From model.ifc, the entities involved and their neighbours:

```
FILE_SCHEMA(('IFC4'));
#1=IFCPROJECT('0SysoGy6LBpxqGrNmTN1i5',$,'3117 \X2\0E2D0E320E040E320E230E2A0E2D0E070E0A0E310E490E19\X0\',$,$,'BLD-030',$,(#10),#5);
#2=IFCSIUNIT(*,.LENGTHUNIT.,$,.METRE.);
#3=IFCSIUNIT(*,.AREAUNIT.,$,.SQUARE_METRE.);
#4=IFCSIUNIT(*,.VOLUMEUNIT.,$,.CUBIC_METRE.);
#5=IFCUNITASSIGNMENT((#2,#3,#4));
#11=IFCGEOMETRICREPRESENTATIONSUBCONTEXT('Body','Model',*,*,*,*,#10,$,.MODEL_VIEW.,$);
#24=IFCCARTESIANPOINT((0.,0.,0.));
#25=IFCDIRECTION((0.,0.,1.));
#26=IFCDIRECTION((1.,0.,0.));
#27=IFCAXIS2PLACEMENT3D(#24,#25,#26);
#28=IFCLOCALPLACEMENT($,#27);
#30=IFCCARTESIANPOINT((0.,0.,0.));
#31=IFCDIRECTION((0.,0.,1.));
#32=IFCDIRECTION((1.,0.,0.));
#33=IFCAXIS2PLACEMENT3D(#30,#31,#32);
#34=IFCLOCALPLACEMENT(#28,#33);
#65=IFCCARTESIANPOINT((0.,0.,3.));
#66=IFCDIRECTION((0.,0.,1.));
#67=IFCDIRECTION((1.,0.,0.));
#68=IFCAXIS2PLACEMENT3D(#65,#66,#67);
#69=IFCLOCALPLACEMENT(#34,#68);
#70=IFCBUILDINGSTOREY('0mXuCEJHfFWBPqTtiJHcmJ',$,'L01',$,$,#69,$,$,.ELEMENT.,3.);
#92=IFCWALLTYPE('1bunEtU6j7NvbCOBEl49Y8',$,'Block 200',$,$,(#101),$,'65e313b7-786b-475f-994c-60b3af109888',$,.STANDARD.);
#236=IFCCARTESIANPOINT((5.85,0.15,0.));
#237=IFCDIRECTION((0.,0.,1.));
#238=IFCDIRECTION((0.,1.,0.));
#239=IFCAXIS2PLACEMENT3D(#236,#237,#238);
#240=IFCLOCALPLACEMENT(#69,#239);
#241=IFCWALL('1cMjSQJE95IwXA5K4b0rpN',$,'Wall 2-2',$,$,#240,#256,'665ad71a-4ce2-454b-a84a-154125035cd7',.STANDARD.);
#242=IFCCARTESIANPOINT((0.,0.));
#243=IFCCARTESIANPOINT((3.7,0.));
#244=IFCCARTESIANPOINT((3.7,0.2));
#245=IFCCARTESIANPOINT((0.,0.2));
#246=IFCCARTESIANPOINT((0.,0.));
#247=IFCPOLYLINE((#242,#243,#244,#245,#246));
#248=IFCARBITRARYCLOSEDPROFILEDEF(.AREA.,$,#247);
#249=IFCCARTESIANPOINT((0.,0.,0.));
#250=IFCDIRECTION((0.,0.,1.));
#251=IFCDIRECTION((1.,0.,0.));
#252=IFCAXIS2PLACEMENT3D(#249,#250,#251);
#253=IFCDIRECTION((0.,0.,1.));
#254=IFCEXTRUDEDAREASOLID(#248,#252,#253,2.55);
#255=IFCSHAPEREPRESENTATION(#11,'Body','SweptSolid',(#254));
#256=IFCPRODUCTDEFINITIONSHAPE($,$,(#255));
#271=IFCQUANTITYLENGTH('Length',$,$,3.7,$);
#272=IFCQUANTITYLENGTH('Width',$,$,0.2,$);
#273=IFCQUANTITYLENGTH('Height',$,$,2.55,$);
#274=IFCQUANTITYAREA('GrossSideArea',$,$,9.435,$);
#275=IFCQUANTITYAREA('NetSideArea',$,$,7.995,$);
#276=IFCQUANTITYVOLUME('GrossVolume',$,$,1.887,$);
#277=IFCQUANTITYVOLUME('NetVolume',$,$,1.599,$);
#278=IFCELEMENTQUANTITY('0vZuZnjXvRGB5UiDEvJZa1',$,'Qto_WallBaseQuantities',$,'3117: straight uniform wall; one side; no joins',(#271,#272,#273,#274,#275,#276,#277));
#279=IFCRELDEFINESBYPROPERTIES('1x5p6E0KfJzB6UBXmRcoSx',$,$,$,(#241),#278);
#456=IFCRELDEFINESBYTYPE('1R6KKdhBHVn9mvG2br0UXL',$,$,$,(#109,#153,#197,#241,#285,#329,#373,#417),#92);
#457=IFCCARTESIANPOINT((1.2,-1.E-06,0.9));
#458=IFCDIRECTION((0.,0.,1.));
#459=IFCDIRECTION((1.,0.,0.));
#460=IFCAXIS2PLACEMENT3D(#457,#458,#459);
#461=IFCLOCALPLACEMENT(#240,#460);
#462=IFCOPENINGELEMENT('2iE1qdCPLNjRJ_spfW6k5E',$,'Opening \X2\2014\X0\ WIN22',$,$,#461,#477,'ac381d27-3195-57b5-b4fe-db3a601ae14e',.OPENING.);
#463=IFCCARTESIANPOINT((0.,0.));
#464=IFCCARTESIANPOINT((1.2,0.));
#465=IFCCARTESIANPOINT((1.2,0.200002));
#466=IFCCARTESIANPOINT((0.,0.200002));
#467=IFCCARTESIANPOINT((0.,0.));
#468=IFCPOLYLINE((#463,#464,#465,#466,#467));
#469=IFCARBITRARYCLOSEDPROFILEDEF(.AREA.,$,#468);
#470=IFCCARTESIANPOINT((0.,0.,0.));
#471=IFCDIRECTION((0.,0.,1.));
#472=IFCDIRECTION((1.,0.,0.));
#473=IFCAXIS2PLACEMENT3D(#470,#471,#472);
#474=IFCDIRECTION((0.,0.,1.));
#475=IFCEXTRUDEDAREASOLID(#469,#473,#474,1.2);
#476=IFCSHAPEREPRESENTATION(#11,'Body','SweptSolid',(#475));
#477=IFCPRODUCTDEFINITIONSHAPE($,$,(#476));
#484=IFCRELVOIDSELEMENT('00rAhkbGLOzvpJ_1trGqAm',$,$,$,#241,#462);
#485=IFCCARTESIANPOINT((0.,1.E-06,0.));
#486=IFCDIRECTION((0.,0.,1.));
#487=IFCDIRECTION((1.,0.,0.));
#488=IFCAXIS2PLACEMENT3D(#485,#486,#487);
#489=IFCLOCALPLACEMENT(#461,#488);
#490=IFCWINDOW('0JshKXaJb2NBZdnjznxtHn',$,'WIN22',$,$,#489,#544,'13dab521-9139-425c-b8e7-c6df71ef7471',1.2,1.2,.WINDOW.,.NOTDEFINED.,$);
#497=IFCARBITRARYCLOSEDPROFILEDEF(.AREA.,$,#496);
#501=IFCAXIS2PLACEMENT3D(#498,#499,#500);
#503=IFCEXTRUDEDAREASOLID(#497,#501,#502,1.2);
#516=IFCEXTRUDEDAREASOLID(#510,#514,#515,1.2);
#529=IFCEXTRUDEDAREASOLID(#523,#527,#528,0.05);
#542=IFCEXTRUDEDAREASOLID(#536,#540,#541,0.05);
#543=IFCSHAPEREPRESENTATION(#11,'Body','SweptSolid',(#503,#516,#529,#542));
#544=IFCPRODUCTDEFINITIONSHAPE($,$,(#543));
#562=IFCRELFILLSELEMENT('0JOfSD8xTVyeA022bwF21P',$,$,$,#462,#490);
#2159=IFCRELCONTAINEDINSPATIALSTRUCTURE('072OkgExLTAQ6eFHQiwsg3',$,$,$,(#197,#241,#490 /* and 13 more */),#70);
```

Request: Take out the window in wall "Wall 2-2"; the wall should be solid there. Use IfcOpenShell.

```python
import ifcopenshell
import ifcopenshell.api.feature
import ifcopenshell.api.pset
import ifcopenshell.api.root
import ifcopenshell.geom
import ifcopenshell.util.element
import ifcopenshell.util.shape
import ifcopenshell.util.unit

model = ifcopenshell.open("model.ifc")
area_scale = ifcopenshell.util.unit.calculate_unit_scale(model, "AREAUNIT")
volume_scale = ifcopenshell.util.unit.calculate_unit_scale(model, "VOLUMEUNIT")
settings = ifcopenshell.geom.settings()


def volume(element):
    """Net volume in cubic metres, openings subtracted."""
    shape = ifcopenshell.geom.create_shape(settings, element)
    return ifcopenshell.util.shape.get_volume(shape.geometry)


window = model.by_id(490)
opening = window.FillsVoids[0].RelatingOpeningElement
wall = opening.VoidsElements[0].RelatingBuildingElement
before = volume(wall)

ifcopenshell.api.root.remove_product(model, product=window)
ifcopenshell.api.feature.remove_feature(model, feature=opening)

after = volume(wall)
thickness = 0.2  # wall thickness in metres

# Update the wall's stored quantities.
qto = model.by_id(ifcopenshell.util.element.get_pset(wall, "Qto_WallBaseQuantities", should_inherit=False)["id"])
ifcopenshell.api.pset.edit_qto(model, qto=qto, properties={
    "NetSideArea": after / thickness / area_scale,
    "NetVolume": after / volume_scale,
})

print(f"wall volume {before:.3f} -> {after:.3f} m3")

model.write("model-out.ifc")
```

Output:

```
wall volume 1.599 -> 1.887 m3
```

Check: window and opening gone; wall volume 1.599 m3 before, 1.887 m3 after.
